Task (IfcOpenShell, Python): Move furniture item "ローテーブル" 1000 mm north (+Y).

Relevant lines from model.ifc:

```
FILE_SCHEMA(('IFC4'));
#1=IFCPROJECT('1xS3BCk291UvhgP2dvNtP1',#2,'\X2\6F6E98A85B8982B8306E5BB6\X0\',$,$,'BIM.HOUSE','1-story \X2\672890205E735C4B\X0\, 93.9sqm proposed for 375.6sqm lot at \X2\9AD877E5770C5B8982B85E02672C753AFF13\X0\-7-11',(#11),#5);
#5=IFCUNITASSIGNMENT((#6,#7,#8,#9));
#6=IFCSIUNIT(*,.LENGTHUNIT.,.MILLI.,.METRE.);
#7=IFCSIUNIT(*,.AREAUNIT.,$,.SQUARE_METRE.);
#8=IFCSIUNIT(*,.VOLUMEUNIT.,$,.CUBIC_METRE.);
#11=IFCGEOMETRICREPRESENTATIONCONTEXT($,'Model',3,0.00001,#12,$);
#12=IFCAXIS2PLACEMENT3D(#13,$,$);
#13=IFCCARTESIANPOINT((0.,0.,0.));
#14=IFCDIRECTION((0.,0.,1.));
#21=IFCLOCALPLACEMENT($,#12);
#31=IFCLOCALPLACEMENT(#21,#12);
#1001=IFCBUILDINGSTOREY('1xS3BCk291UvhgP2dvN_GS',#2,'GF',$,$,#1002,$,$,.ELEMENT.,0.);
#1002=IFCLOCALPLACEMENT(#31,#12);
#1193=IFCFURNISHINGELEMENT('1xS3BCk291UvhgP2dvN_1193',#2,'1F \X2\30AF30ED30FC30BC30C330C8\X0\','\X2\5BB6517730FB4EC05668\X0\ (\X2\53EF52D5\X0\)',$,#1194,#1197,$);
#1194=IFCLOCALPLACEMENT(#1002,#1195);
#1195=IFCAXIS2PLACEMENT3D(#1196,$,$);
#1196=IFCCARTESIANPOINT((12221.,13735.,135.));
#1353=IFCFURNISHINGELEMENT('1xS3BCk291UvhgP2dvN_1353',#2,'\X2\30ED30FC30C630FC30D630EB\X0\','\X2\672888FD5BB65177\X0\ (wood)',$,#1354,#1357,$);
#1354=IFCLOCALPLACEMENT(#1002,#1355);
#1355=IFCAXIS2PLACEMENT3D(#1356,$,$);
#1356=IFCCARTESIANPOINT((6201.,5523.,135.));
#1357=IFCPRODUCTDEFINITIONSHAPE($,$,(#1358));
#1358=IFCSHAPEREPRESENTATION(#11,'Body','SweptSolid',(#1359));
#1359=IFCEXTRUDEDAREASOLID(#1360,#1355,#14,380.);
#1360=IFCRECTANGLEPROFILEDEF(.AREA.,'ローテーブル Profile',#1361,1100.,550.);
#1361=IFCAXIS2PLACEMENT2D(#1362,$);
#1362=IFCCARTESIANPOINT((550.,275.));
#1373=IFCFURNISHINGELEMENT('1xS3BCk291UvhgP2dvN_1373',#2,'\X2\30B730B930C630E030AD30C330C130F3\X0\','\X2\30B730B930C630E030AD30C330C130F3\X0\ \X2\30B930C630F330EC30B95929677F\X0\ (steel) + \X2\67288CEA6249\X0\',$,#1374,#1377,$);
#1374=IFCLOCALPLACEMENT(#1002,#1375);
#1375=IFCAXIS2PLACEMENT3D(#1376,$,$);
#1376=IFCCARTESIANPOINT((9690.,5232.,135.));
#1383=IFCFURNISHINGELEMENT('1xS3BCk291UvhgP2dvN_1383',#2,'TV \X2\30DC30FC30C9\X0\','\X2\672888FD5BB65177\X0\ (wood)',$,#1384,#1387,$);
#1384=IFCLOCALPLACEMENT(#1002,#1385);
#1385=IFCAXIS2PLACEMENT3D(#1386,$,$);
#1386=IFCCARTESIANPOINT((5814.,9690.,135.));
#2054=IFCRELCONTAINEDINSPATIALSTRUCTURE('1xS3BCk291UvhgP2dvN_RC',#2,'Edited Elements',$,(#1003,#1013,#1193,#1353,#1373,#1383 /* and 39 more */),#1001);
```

```python
import ifcopenshell
import ifcopenshell.api.geometry
import ifcopenshell.util.placement
import ifcopenshell.util.unit

model = ifcopenshell.open("model.ifc")
unit_scale = ifcopenshell.util.unit.calculate_unit_scale(model)

item = model.by_guid("1xS3BCk291UvhgP2dvN_1353")
matrix = ifcopenshell.util.placement.get_local_placement(item.ObjectPlacement)
matrix[1, 3] += 1 / unit_scale
ifcopenshell.api.geometry.edit_object_placement(model, product=item, matrix=matrix, is_si=False)

print(ifcopenshell.util.placement.get_local_placement(item.ObjectPlacement).round(3) + 0.0)

model.write("model_updated.ifc")
```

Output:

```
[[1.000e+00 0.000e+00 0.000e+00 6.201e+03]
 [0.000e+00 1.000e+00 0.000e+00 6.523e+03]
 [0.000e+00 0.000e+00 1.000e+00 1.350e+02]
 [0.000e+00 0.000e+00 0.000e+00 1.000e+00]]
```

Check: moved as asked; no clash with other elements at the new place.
